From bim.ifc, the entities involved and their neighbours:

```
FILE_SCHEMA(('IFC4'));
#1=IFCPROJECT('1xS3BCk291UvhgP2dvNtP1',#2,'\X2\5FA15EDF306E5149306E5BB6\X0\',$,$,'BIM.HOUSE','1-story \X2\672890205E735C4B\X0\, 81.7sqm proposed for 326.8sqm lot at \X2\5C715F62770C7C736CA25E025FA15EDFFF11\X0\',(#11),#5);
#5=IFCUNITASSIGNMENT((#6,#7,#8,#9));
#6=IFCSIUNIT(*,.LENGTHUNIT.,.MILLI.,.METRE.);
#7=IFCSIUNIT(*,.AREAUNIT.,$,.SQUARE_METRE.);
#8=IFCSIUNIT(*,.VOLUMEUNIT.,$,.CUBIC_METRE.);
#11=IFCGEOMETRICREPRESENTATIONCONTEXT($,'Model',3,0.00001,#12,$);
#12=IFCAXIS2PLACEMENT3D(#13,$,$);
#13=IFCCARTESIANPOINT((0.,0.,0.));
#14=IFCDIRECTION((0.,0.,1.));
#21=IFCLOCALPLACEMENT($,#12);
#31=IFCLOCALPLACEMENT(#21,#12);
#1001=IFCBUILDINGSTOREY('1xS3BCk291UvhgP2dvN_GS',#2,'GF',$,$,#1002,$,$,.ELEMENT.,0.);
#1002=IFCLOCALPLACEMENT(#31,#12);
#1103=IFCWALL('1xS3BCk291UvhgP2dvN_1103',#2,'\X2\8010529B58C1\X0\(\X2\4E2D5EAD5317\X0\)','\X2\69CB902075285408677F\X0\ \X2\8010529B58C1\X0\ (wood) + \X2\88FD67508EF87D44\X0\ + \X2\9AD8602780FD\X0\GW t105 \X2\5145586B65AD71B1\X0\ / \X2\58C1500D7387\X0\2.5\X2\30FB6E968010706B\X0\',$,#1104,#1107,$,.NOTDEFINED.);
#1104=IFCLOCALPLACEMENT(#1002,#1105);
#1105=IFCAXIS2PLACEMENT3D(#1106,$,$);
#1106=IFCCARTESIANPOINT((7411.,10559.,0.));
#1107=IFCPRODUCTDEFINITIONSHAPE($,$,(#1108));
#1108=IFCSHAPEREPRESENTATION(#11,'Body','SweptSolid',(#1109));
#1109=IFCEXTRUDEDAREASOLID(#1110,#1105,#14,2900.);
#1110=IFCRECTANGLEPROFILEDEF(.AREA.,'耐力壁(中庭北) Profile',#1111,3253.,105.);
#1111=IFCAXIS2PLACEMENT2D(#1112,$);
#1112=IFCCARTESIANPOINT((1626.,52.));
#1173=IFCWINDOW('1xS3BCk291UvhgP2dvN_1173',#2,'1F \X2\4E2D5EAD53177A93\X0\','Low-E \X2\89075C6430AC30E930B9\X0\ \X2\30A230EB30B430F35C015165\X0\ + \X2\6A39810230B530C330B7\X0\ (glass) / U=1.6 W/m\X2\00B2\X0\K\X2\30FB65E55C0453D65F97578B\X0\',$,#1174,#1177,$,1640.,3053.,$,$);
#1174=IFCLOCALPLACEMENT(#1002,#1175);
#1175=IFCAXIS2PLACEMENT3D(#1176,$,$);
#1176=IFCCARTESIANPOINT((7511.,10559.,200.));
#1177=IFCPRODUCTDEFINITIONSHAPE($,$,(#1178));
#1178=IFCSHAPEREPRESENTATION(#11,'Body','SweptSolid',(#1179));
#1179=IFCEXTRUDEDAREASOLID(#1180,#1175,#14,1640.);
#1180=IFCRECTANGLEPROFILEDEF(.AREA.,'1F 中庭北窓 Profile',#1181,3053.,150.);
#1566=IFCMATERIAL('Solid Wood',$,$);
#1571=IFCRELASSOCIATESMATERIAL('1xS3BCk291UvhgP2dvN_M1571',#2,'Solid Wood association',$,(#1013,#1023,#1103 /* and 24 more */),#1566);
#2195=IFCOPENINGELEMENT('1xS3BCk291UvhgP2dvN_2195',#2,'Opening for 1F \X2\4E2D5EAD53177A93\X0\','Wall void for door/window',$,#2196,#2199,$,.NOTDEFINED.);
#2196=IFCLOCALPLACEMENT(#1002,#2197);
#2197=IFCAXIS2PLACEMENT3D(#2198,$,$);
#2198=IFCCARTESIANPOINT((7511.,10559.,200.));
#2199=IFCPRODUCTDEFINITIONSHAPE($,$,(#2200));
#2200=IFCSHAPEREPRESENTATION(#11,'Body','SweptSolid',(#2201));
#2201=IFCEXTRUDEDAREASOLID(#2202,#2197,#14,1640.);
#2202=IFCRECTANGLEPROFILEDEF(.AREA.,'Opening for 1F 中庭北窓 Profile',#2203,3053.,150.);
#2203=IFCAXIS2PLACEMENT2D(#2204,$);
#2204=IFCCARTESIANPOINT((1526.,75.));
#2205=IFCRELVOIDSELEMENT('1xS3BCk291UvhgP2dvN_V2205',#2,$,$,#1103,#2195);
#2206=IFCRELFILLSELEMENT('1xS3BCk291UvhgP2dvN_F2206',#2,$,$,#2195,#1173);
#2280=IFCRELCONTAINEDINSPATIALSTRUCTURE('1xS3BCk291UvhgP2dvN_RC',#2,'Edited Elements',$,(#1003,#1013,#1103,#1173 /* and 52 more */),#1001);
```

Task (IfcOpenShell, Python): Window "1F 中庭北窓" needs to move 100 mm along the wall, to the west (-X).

```python
import ifcopenshell
import ifcopenshell.api.geometry
import ifcopenshell.util.placement
import ifcopenshell.util.unit

model = ifcopenshell.open("bim.ifc")
unit_scale = ifcopenshell.util.unit.calculate_unit_scale(model)

window = model.by_id(1173)
opening = window.FillsVoids[0].RelatingOpeningElement
wall = opening.VoidsElements[0].RelatingBuildingElement

wall_matrix = ifcopenshell.util.placement.get_local_placement(wall.ObjectPlacement)
shift = wall_matrix[:3, 0] * -0.1 / unit_scale
before = ifcopenshell.util.placement.get_local_placement(window.ObjectPlacement)[:3, 3].copy()

# The window is not placed relative to its opening, so move both.
for product in (opening, window):
    matrix = ifcopenshell.util.placement.get_local_placement(product.ObjectPlacement)
    matrix[:3, 3] += shift
    ifcopenshell.api.geometry.edit_object_placement(model, product=product, matrix=matrix, is_si=False)

after = ifcopenshell.util.placement.get_local_placement(window.ObjectPlacement)[:3, 3]
print("window moved by", (after - before).round(3) + 0.0)

model.write("bim_rev.ifc")
```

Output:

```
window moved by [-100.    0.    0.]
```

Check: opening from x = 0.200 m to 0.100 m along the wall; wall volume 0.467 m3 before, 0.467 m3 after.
